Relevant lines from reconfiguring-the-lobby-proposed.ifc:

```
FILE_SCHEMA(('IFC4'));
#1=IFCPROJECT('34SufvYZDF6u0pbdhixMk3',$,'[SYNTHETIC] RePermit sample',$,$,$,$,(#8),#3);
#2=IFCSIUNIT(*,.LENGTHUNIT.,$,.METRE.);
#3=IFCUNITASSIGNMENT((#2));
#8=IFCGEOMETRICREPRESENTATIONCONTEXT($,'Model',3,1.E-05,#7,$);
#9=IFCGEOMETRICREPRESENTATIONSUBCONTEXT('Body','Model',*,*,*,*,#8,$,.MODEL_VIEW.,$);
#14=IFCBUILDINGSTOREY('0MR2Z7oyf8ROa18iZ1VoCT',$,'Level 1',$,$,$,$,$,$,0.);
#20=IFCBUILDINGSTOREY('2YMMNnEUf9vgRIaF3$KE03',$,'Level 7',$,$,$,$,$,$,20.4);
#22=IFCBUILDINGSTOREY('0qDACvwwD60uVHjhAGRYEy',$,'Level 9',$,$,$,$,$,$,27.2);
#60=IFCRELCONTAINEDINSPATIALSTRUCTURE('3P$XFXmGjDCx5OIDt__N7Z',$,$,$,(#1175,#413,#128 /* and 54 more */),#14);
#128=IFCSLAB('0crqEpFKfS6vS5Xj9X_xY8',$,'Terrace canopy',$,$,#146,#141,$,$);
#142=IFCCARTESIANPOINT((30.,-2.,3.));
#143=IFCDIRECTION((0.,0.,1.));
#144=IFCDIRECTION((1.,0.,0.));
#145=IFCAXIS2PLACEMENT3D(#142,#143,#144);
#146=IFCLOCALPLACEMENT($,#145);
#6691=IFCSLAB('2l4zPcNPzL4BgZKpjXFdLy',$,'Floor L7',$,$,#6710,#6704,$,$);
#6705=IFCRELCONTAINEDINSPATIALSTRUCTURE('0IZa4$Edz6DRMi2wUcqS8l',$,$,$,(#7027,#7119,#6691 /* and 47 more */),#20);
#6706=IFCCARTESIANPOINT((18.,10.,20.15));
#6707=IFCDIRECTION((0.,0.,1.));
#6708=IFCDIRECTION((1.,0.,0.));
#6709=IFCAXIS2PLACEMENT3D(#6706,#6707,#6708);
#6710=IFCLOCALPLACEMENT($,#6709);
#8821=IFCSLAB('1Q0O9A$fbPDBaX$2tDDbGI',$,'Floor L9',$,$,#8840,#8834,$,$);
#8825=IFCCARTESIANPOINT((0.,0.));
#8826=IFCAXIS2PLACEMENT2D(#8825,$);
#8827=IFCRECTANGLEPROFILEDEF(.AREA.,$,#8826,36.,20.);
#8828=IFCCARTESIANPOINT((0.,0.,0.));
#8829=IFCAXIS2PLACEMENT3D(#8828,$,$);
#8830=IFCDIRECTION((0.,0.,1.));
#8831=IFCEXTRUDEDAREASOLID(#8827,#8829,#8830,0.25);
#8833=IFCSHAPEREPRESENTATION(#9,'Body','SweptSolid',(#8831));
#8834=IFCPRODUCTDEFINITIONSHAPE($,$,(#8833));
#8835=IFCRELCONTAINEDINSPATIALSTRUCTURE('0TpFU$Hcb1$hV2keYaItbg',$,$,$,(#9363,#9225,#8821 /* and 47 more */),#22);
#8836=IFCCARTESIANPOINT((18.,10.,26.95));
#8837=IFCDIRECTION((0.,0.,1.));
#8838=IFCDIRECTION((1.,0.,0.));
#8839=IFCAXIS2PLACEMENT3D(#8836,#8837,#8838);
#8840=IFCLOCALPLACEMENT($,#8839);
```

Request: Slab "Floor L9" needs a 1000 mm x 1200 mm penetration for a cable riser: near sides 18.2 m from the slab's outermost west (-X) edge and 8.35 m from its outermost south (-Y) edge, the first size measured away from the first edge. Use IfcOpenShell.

```python
import numpy as np
import ifcopenshell
import ifcopenshell.api.feature
import ifcopenshell.api.geometry
import ifcopenshell.api.root
import ifcopenshell.geom
import ifcopenshell.util.placement
import ifcopenshell.util.representation
import ifcopenshell.util.shape
import ifcopenshell.util.unit

model = ifcopenshell.open("reconfiguring-the-lobby-proposed.ifc")
unit_scale = ifcopenshell.util.unit.calculate_unit_scale(model)
settings = ifcopenshell.geom.settings()


def volume(element):
    """Net volume in cubic metres, openings subtracted."""
    shape = ifcopenshell.geom.create_shape(settings, element)
    return ifcopenshell.util.shape.get_volume(shape.geometry)


slab = model.by_guid("1Q0O9A$fbPDBaX$2tDDbGI")
before = volume(slab)

# Extent in the slab's own axes, in metres. The edges named are its -X and -Y sides.
slab_shape = ifcopenshell.geom.create_shape(settings, slab)
vertices = ifcopenshell.util.shape.get_vertices(slab_shape.geometry)
x_min, y_min, bottom = vertices.min(axis=0)
top = vertices[:, 2].max()

opening = ifcopenshell.api.root.create_entity(model, ifc_class="IfcOpeningElement", name="Cable riser opening", predefined_type="OPENING")
context = ifcopenshell.util.representation.get_context(model, "Model", "Body", "MODEL_VIEW")
width, depth = 1, 1.2
outline = [(0.0, 0.0), (width, 0.0), (width, depth), (0.0, depth), (0.0, 0.0)]
# Overshoot both faces by 50 mm so the cut is clean.
shape = ifcopenshell.api.geometry.add_slab_representation(
    model, context=context, depth=top - bottom + 0.1, polyline=outline
)
ifcopenshell.api.geometry.assign_representation(model, product=opening, representation=shape)

matrix = ifcopenshell.util.placement.get_local_placement(slab.ObjectPlacement)
matrix[:, 3] = matrix @ np.append(np.array([x_min + 18.2, y_min + 8.35, bottom - 0.05]) / unit_scale, 1.0)
ifcopenshell.api.geometry.edit_object_placement(model, product=opening, matrix=matrix, is_si=False)
ifcopenshell.api.feature.add_feature(model, feature=opening, element=slab)

after = volume(slab)

print(f"slab volume {before:.3f} -> {after:.3f} m3")

model.write("reconfiguring-the-lobby-proposed_rev.ifc")
```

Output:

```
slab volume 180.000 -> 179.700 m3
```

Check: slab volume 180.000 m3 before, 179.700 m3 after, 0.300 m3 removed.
